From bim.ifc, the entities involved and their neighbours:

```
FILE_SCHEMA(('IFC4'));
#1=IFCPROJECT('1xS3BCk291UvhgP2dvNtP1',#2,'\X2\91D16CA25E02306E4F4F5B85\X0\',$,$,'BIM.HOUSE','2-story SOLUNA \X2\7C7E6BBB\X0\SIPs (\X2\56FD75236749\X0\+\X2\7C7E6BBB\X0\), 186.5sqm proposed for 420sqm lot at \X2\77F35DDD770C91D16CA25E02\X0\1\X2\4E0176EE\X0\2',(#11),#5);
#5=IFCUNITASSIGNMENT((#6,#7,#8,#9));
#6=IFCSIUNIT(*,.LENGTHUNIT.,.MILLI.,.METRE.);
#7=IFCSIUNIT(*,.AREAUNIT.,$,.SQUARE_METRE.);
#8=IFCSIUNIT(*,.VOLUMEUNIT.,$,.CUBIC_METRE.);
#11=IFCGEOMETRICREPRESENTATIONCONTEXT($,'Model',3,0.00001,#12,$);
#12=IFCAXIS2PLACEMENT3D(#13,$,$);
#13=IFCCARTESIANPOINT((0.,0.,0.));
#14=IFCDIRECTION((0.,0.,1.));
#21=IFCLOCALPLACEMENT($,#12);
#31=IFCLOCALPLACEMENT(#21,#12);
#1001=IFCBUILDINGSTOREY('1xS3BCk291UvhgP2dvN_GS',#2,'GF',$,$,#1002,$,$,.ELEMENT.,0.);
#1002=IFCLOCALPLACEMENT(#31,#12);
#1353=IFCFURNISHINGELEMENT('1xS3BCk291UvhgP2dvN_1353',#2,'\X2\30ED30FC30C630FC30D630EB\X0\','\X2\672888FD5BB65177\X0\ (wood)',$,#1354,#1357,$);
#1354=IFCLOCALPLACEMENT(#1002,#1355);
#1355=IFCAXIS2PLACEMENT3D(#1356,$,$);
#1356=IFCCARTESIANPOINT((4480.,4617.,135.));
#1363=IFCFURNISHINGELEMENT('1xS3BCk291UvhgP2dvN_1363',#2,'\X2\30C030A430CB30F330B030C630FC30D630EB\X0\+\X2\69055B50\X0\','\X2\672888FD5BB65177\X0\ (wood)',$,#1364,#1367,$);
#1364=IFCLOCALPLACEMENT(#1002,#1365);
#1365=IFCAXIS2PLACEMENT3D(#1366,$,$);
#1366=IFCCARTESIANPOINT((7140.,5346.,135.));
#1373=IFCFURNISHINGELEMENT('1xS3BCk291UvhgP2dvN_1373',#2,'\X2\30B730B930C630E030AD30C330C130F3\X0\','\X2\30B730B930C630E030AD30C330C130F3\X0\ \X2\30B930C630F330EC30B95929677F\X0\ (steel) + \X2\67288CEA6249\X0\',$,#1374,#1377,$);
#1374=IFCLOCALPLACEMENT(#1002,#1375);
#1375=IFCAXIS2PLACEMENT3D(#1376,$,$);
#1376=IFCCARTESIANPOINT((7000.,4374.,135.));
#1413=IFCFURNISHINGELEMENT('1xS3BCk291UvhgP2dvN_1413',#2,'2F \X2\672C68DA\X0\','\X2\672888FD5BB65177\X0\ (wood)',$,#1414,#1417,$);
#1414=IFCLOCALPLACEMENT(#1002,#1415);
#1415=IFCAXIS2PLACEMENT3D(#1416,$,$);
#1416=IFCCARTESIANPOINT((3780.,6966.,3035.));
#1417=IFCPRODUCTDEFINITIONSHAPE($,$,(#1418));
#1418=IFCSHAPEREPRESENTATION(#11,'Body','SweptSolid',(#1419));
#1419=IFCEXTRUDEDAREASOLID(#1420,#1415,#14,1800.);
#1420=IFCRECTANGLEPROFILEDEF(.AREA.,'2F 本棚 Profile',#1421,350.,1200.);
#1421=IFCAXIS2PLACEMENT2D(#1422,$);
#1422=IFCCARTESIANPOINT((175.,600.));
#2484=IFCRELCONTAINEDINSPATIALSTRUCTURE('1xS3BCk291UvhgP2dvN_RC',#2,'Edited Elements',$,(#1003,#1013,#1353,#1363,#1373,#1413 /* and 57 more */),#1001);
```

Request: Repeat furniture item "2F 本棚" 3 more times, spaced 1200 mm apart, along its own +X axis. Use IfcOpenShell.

```python
import ifcopenshell
import ifcopenshell.api.geometry
import ifcopenshell.api.root
import ifcopenshell.util.element
import ifcopenshell.util.placement

model = ifcopenshell.open("bim.ifc")


def reuse_history(source, copy):
    """copy_class also copies each property set's owner history, people and application; keep the originals."""
    for rel in copy.IsDefinedBy:
        if rel.is_a("IfcRelDefinesByProperties") and (history := rel.RelatingPropertyDefinition.OwnerHistory):
            rel.RelatingPropertyDefinition.OwnerHistory = source.OwnerHistory
            ifcopenshell.util.element.remove_deep2(model, history)


source = model.by_id(1413)
base = ifcopenshell.util.placement.get_local_placement(source.ObjectPlacement)
step = base[:3, 0] * 1200.0

for i in range(1, 4):
    copy = ifcopenshell.api.root.copy_class(model, product=source)
    copy.Representation = ifcopenshell.util.element.copy_deep(
        model, source.Representation, exclude=["IfcGeometricRepresentationContext", "IfcRepresentationMap"]
    )
    reuse_history(source, copy)
    matrix = base.copy()
    matrix[:3, 3] += i * step
    print("added at", matrix[:3, 3].round(3) + 0.0)
    ifcopenshell.api.geometry.edit_object_placement(model, product=copy, matrix=matrix, is_si=False)

model.write("bim_rev.ifc")
```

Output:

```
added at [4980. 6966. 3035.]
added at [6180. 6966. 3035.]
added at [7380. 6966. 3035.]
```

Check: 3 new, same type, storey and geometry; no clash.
